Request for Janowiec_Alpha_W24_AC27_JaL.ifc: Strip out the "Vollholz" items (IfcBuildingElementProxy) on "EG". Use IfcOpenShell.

First a look at what the model holds.

```python
import ifcopenshell
import ifcopenshell.util.element

model = ifcopenshell.open("Janowiec_Alpha_W24_AC27_JaL.ifc")
print(model.schema)
storey = next(s for s in model.by_type("IfcBuildingStorey") if s.Name == "EG")
proxies = [e for e in ifcopenshell.util.element.get_decomposition(storey) if e.is_a("IfcBuildingElementProxy")]
seen = {}
for e in proxies:
    element_type = ifcopenshell.util.element.get_type(e)
    name = element_type.Name if element_type not in (None, e) else None
    seen[name] = seen.get(name, 0) + 1
for name, count in sorted(seen.items(), key=str):
    print(count, "x", name)
```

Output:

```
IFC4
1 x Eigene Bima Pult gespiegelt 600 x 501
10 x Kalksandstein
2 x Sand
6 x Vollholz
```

```python
import ifcopenshell
import ifcopenshell.api.root
import ifcopenshell.util.element

model = ifcopenshell.open("Janowiec_Alpha_W24_AC27_JaL.ifc")

storey = next(s for s in model.by_type("IfcBuildingStorey") if s.Name == "EG")
proxies = [e for e in ifcopenshell.util.element.get_decomposition(storey) if e.is_a("IfcBuildingElementProxy")]
targets = [e for e in proxies if (t := ifcopenshell.util.element.get_type(e)) not in (None, e) and t.Name == "Vollholz"]

for e in targets:
    ifcopenshell.api.root.remove_product(model, product=e)
print(len(targets), "removed")

model.write("Janowiec_Alpha_W24_AC27_JaL_updated.ifc")
```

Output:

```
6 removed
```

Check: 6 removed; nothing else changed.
